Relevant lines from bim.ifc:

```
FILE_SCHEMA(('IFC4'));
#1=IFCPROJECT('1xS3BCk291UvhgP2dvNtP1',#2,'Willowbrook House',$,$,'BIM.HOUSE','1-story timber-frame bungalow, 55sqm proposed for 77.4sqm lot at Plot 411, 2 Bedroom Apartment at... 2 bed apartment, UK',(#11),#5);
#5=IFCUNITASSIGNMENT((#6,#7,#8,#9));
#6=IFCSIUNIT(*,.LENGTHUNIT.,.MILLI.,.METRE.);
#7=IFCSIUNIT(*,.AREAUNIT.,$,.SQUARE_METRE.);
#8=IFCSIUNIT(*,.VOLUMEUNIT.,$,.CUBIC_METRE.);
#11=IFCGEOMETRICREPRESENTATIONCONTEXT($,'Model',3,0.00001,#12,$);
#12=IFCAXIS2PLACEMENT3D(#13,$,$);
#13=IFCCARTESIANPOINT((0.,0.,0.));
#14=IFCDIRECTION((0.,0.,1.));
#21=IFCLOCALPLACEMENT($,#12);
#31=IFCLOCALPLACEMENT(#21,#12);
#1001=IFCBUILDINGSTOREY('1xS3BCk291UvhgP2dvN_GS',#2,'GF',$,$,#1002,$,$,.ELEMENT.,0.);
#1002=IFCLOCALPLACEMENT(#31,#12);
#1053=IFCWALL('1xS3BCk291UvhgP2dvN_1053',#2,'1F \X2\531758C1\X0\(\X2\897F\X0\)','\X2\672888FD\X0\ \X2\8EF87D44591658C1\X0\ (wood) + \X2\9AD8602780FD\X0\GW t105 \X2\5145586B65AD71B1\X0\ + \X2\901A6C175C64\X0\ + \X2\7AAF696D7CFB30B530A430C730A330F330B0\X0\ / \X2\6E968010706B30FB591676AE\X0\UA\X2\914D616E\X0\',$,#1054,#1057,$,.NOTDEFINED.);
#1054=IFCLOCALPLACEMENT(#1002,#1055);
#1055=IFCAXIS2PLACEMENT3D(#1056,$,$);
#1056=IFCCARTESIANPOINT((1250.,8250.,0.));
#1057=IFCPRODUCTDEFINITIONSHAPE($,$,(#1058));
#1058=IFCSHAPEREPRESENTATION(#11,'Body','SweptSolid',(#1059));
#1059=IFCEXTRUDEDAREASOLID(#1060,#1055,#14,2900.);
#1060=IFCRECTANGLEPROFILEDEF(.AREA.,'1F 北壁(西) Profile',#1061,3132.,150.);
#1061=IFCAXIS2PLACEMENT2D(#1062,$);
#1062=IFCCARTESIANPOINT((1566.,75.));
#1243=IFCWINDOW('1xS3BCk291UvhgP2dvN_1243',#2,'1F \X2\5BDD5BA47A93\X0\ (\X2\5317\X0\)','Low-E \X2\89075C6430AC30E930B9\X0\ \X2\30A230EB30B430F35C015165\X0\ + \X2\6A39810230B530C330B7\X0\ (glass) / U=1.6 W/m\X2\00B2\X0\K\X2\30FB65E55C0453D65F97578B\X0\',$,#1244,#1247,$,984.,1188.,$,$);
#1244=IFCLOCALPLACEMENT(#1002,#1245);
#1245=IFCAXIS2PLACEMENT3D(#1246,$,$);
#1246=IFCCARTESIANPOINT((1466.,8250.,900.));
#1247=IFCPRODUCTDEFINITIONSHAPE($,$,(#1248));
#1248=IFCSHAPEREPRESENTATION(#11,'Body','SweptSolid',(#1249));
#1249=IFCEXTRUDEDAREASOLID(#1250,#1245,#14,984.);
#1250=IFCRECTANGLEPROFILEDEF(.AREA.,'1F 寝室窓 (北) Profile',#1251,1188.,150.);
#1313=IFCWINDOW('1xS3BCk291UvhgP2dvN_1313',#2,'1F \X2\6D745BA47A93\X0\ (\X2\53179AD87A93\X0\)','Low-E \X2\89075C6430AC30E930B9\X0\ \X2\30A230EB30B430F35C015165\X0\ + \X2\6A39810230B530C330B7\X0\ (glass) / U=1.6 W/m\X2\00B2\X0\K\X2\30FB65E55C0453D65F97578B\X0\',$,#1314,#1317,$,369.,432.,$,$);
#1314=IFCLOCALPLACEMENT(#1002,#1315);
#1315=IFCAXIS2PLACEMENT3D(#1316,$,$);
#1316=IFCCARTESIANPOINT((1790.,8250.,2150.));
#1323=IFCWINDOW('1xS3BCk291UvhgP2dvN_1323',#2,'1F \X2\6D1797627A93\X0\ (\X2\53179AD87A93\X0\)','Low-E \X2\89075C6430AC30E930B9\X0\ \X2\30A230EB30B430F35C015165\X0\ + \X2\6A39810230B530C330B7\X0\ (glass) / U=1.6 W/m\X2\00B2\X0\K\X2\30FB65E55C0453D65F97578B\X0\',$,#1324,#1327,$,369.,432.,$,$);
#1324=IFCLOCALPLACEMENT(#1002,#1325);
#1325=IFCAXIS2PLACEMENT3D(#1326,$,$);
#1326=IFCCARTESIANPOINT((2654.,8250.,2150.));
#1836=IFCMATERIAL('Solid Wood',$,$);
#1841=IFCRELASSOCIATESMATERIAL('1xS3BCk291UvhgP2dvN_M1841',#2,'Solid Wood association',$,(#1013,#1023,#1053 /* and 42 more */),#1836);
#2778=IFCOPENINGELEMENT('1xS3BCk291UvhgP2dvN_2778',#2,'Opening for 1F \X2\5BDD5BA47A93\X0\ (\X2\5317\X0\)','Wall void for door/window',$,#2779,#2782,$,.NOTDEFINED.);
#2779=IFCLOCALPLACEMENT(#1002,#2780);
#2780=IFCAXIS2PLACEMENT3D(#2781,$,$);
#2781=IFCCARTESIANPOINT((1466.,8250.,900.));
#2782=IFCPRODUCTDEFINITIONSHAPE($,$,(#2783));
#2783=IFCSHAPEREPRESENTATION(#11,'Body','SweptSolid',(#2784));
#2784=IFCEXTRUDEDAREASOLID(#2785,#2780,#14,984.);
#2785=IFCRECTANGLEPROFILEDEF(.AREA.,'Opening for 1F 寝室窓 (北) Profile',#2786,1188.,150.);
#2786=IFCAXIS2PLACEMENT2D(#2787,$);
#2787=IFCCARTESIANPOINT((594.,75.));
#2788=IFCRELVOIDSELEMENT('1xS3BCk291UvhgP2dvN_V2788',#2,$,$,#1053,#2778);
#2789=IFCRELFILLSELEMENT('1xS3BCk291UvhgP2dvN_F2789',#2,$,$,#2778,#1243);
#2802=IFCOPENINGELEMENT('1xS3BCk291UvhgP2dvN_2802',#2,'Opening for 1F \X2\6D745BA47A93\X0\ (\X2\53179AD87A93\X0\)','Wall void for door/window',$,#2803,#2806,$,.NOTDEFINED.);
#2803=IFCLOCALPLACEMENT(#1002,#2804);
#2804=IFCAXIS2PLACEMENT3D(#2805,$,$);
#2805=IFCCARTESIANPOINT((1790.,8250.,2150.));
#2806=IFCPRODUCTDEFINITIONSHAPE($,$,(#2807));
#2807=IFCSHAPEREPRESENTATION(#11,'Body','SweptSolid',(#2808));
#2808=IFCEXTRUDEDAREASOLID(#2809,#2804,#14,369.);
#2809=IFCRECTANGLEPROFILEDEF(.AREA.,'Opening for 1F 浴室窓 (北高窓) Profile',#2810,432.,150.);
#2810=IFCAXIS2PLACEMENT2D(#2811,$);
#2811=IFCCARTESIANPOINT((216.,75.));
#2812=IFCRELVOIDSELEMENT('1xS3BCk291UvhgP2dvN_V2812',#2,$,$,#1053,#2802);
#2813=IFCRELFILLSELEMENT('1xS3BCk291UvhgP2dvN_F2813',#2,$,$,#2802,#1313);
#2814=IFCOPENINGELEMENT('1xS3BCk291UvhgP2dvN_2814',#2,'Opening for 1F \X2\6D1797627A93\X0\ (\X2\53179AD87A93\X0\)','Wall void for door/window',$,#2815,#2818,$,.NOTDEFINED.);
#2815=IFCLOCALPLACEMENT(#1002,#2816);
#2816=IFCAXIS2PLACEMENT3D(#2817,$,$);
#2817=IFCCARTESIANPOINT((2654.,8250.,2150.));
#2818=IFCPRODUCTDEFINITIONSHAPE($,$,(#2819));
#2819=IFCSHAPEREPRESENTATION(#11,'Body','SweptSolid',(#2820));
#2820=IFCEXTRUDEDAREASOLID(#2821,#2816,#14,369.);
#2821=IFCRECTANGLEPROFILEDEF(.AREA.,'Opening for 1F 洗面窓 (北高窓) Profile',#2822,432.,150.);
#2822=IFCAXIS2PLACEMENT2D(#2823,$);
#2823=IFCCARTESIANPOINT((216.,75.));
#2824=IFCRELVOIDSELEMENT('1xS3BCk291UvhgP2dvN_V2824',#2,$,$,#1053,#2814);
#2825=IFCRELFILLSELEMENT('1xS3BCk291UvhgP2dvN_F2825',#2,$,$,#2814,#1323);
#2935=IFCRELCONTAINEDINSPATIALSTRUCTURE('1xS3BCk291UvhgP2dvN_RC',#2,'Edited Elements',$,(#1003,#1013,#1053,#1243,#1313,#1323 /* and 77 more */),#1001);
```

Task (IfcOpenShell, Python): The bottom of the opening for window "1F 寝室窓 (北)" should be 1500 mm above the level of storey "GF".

```python
import numpy as np
import ifcopenshell
import ifcopenshell.api.geometry
import ifcopenshell.geom
import ifcopenshell.util.element
import ifcopenshell.util.placement
import ifcopenshell.util.shape
import ifcopenshell.util.unit

model = ifcopenshell.open("bim.ifc")
unit_scale = ifcopenshell.util.unit.calculate_unit_scale(model)

window = model.by_id(1243)
opening = window.FillsVoids[0].RelatingOpeningElement
storey = ifcopenshell.util.element.get_container(window, ifc_class="IfcBuildingStorey")
level = ifcopenshell.util.placement.get_local_placement(storey.ObjectPlacement)[2, 3]

# The opening's origin need not be at the sill, so measure its lowest point.
shape = ifcopenshell.geom.create_shape(ifcopenshell.geom.settings(), opening)
bottom = ifcopenshell.util.shape.get_shape_bottom_elevation(shape, shape.geometry) / unit_scale
dz = level + 1.5 / unit_scale - bottom

shift = np.array([0.0, 0.0, dz])
# The window is not placed relative to its opening, so move both.
for product in (opening, window):
    matrix = ifcopenshell.util.placement.get_local_placement(product.ObjectPlacement)
    matrix[:3, 3] += shift
    ifcopenshell.api.geometry.edit_object_placement(model, product=product, matrix=matrix, is_si=False)

print(f"moved by {dz * unit_scale:+.3f} m")

model.write("bim_rev.ifc")
```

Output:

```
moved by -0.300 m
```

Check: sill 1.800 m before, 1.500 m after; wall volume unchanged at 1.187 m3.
